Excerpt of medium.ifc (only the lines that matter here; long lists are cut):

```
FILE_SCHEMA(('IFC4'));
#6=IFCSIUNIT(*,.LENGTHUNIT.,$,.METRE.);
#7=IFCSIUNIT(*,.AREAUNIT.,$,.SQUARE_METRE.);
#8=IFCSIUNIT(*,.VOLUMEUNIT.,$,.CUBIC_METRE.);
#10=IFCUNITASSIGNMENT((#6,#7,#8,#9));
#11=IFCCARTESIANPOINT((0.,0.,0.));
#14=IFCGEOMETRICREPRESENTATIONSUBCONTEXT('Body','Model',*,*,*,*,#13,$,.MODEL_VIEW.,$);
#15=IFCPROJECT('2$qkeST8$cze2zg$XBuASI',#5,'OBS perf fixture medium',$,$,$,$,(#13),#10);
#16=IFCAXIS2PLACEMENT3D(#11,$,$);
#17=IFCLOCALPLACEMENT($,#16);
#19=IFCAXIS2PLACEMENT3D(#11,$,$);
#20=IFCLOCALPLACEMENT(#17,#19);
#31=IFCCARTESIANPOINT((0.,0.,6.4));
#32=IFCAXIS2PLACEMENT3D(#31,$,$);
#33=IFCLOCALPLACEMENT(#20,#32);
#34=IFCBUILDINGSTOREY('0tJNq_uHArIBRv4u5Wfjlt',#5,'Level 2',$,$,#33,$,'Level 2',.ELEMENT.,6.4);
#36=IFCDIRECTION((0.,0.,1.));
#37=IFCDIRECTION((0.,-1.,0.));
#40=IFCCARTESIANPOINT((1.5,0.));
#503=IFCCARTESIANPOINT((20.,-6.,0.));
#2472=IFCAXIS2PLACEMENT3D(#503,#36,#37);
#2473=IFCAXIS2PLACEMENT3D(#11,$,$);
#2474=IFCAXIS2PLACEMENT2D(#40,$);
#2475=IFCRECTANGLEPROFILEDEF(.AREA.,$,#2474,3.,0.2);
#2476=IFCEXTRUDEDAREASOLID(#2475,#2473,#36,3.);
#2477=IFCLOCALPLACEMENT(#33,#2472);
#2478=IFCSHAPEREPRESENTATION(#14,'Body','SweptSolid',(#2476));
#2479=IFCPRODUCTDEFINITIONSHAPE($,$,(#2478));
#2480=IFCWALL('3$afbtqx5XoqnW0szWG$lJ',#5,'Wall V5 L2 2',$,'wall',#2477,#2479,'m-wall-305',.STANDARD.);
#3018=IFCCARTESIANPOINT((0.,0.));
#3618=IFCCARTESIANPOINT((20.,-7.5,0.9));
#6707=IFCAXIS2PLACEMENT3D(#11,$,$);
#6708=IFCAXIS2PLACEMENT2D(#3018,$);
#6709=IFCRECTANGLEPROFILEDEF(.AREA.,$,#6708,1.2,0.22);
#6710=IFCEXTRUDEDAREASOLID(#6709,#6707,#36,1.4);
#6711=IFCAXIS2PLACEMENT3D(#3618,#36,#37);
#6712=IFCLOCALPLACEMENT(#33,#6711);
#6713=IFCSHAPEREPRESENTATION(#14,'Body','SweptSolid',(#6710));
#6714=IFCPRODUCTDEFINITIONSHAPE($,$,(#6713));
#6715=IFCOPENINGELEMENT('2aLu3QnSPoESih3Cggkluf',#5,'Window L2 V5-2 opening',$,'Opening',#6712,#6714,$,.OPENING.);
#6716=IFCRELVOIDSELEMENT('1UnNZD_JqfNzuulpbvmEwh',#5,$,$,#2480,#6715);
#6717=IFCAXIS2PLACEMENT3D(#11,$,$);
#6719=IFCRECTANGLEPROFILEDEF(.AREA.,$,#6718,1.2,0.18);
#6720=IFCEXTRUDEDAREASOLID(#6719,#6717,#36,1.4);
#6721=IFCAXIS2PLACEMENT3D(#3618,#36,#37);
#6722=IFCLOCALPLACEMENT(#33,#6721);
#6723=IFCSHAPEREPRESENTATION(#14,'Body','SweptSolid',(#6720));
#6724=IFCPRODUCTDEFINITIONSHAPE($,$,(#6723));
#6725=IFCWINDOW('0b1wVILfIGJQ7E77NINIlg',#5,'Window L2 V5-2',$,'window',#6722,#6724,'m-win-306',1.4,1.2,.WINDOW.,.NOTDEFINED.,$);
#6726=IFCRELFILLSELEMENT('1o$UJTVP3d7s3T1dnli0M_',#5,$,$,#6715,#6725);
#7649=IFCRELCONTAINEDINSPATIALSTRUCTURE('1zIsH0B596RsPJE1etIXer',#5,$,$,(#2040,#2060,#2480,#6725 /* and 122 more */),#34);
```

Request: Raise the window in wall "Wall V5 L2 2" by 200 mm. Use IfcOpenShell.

```python
import numpy as np
import ifcopenshell
import ifcopenshell.api.geometry
import ifcopenshell.util.placement
import ifcopenshell.util.unit

model = ifcopenshell.open("medium.ifc")
unit_scale = ifcopenshell.util.unit.calculate_unit_scale(model)

window = model.by_guid("0b1wVILfIGJQ7E77NINIlg")
opening = window.FillsVoids[0].RelatingOpeningElement
dz = 0.2 / unit_scale

shift = np.array([0.0, 0.0, dz])
# The window is not placed relative to its opening, so move both.
for product in (opening, window):
    matrix = ifcopenshell.util.placement.get_local_placement(product.ObjectPlacement)
    matrix[:3, 3] += shift
    ifcopenshell.api.geometry.edit_object_placement(model, product=product, matrix=matrix, is_si=False)

print(f"moved by {dz * unit_scale:+.3f} m")

model.write("medium_rev.ifc")
```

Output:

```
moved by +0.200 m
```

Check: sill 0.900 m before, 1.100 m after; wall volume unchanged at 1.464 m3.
